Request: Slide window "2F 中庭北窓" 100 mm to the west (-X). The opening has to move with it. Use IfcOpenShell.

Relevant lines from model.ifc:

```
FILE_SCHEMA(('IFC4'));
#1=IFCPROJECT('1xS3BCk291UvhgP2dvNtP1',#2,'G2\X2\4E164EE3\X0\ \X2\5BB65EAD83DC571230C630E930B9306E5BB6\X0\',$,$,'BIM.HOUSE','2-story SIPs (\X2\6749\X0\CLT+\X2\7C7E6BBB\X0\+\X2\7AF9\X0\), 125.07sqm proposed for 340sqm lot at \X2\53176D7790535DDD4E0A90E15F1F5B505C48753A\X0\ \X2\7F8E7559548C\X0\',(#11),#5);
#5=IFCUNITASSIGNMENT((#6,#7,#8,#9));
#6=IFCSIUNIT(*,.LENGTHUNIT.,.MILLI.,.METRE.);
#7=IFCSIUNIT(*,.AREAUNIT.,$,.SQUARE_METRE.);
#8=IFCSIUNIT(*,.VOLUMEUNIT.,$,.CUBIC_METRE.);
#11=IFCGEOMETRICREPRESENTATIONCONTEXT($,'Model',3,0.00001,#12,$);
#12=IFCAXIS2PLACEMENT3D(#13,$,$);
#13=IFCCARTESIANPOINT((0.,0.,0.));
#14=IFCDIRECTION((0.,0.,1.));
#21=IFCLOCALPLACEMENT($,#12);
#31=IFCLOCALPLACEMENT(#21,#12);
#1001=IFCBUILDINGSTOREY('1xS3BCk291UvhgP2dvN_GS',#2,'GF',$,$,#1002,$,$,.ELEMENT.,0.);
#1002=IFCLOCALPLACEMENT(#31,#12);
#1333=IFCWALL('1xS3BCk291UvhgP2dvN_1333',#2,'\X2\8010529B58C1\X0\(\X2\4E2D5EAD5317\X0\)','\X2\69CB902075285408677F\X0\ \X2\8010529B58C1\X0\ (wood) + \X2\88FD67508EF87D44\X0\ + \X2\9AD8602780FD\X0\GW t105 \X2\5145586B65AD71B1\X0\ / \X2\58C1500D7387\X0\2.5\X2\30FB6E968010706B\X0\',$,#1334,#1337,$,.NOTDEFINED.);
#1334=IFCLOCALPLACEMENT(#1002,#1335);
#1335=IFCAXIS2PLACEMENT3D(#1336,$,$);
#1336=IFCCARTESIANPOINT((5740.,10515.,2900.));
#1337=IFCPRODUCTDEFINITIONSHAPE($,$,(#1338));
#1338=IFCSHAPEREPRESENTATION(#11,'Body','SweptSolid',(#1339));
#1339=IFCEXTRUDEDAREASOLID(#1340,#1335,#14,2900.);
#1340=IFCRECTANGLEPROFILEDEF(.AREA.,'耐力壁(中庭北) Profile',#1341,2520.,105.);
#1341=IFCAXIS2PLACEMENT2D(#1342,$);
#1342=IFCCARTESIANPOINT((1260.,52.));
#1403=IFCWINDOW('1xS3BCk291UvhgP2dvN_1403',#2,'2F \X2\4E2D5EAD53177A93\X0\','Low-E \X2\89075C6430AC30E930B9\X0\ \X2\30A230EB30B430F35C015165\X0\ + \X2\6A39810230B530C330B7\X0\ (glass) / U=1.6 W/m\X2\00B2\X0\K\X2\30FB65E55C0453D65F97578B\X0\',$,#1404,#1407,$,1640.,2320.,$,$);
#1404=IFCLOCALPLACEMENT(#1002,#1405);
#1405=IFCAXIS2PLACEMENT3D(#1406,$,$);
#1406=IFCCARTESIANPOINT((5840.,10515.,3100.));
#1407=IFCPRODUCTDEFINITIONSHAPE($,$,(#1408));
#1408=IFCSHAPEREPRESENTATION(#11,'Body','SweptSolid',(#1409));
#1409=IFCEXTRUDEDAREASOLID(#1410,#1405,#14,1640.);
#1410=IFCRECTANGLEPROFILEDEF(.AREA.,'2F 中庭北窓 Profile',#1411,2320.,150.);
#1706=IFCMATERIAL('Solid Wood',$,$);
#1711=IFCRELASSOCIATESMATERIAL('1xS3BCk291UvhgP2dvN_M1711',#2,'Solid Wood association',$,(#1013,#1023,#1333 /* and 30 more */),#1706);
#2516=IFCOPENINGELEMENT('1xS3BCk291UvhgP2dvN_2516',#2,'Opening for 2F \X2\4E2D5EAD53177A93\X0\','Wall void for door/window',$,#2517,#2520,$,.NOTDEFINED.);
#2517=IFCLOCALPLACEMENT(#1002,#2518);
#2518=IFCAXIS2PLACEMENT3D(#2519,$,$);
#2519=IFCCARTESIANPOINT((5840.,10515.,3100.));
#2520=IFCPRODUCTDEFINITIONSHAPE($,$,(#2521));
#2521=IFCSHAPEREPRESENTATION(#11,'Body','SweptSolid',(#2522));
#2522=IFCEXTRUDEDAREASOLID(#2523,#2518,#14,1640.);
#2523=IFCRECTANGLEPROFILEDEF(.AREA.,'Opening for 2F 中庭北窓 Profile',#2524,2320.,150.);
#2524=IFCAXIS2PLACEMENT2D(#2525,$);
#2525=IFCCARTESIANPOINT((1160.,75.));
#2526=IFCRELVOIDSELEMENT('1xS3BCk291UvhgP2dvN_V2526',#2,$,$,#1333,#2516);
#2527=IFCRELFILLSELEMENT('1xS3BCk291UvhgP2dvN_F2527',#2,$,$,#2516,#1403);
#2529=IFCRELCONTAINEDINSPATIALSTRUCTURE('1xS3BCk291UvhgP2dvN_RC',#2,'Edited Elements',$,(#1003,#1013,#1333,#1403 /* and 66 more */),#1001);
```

```python
import ifcopenshell
import ifcopenshell.api.geometry
import ifcopenshell.util.placement
import ifcopenshell.util.unit

model = ifcopenshell.open("model.ifc")
unit_scale = ifcopenshell.util.unit.calculate_unit_scale(model)

window = model.by_guid("1xS3BCk291UvhgP2dvN_1403")
opening = window.FillsVoids[0].RelatingOpeningElement
wall = opening.VoidsElements[0].RelatingBuildingElement

wall_matrix = ifcopenshell.util.placement.get_local_placement(wall.ObjectPlacement)
shift = wall_matrix[:3, 0] * -0.1 / unit_scale
before = ifcopenshell.util.placement.get_local_placement(window.ObjectPlacement)[:3, 3].copy()

# The window is not placed relative to its opening, so move both.
for product in (opening, window):
    matrix = ifcopenshell.util.placement.get_local_placement(product.ObjectPlacement)
    matrix[:3, 3] += shift
    ifcopenshell.api.geometry.edit_object_placement(model, product=product, matrix=matrix, is_si=False)

after = ifcopenshell.util.placement.get_local_placement(window.ObjectPlacement)[:3, 3]
print("window moved by", (after - before).round(3) + 0.0)

model.write("model_v2.ifc")
```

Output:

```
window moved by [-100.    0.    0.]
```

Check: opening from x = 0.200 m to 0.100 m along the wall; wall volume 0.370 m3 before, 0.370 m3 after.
